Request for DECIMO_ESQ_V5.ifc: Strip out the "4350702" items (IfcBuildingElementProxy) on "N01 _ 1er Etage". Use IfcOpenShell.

First a look at what the model holds.

```python
import ifcopenshell
import ifcopenshell.util.element

model = ifcopenshell.open("DECIMO_ESQ_V5.ifc")
print(model.schema)
storey = next(s for s in model.by_type("IfcBuildingStorey") if s.Name == "N01 _ 1er Etage")
proxies = [e for e in ifcopenshell.util.element.get_decomposition(storey) if e.is_a("IfcBuildingElementProxy")]
seen = {}
for e in proxies:
    element_type = ifcopenshell.util.element.get_type(e)
    name = element_type.Name if element_type not in (None, e) else None
    seen[name] = seen.get(name, 0) + 1
for name, count in sorted(seen.items(), key=str):
    print(count, "x", name)
```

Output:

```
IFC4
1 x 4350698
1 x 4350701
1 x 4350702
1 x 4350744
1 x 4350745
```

```python
import ifcopenshell
import ifcopenshell.api.root
import ifcopenshell.util.element

model = ifcopenshell.open("DECIMO_ESQ_V5.ifc")

storey = next(s for s in model.by_type("IfcBuildingStorey") if s.Name == "N01 _ 1er Etage")
proxies = [e for e in ifcopenshell.util.element.get_decomposition(storey) if e.is_a("IfcBuildingElementProxy")]
targets = [e for e in proxies if (t := ifcopenshell.util.element.get_type(e)) not in (None, e) and t.Name == "4350702"]

for e in targets:
    ifcopenshell.api.root.remove_product(model, product=e)
print(len(targets), "removed")

model.write("DECIMO_ESQ_V5_rev.ifc")
```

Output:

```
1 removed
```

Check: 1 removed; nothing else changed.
